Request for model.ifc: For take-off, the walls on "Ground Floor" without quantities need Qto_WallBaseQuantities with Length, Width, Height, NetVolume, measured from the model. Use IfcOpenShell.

First a look at what the model holds.

```python
import ifcopenshell
import ifcopenshell.util.element
import ifcopenshell.util.unit

model = ifcopenshell.open("model.ifc")
print(model.schema)
for unit_type in ("LENGTHUNIT", "AREAUNIT", "VOLUMEUNIT"):
    print(unit_type, ifcopenshell.util.unit.calculate_unit_scale(model, unit_type))
storey = next(s for s in model.by_type("IfcBuildingStorey") if s.Name == "Ground Floor")
walls = [e for e in ifcopenshell.util.element.get_decomposition(storey) if e.is_a("IfcWall")]
for e in sorted(walls, key=lambda e: e.id()):
    print(e.id(), e.is_a(), e.Name, list(ifcopenshell.util.element.get_psets(e, qtos_only=True)), sep=" | ")
```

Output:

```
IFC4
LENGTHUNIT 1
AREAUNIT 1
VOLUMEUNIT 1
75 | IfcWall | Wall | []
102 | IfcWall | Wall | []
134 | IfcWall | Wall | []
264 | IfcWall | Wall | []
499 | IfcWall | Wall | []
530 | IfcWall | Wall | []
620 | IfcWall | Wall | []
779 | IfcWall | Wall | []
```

```python
import ifcopenshell
import ifcopenshell.api.pset
import ifcopenshell.geom
import ifcopenshell.util.element
import ifcopenshell.util.shape
import ifcopenshell.util.unit

model = ifcopenshell.open("model.ifc")
unit_scale = ifcopenshell.util.unit.calculate_unit_scale(model)
volume_scale = ifcopenshell.util.unit.calculate_unit_scale(model, "VOLUMEUNIT")
settings = ifcopenshell.geom.settings()

storey = next(s for s in model.by_type("IfcBuildingStorey") if s.Name == "Ground Floor")
walls = [e for e in ifcopenshell.util.element.get_decomposition(storey) if e.is_a("IfcWall")]

for e in sorted(walls, key=lambda e: e.id()):
    if ifcopenshell.util.element.get_psets(e, qtos_only=True, should_inherit=False):
        continue
    # Geometry comes back in metres, in the element's own axes.
    shape = ifcopenshell.geom.create_shape(settings, e)
    values = {
        "Length": ifcopenshell.util.shape.get_x(shape.geometry) / unit_scale,
        "Width": ifcopenshell.util.shape.get_y(shape.geometry) / unit_scale,
        "Height": ifcopenshell.util.shape.get_z(shape.geometry) / unit_scale,
        "NetVolume": ifcopenshell.util.shape.get_volume(shape.geometry) / volume_scale,
    }
    qto = ifcopenshell.api.pset.add_qto(model, product=e, name="Qto_WallBaseQuantities")
    ifcopenshell.api.pset.edit_qto(model, qto=qto, properties=values)
    print(e.id(), {k: round(v, 3) for k, v in values.items()})

model.write("model_v2.ifc")
```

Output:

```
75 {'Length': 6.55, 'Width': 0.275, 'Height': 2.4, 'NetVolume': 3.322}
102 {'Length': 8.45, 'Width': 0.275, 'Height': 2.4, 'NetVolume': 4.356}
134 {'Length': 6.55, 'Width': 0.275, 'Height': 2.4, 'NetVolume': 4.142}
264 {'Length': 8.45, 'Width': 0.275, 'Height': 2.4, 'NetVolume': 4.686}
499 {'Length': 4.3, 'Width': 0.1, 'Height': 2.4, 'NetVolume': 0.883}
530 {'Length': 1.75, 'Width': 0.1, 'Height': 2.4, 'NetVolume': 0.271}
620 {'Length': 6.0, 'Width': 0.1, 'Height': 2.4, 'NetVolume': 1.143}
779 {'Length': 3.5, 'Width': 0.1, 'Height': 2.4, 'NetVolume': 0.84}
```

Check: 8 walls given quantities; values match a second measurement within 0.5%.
